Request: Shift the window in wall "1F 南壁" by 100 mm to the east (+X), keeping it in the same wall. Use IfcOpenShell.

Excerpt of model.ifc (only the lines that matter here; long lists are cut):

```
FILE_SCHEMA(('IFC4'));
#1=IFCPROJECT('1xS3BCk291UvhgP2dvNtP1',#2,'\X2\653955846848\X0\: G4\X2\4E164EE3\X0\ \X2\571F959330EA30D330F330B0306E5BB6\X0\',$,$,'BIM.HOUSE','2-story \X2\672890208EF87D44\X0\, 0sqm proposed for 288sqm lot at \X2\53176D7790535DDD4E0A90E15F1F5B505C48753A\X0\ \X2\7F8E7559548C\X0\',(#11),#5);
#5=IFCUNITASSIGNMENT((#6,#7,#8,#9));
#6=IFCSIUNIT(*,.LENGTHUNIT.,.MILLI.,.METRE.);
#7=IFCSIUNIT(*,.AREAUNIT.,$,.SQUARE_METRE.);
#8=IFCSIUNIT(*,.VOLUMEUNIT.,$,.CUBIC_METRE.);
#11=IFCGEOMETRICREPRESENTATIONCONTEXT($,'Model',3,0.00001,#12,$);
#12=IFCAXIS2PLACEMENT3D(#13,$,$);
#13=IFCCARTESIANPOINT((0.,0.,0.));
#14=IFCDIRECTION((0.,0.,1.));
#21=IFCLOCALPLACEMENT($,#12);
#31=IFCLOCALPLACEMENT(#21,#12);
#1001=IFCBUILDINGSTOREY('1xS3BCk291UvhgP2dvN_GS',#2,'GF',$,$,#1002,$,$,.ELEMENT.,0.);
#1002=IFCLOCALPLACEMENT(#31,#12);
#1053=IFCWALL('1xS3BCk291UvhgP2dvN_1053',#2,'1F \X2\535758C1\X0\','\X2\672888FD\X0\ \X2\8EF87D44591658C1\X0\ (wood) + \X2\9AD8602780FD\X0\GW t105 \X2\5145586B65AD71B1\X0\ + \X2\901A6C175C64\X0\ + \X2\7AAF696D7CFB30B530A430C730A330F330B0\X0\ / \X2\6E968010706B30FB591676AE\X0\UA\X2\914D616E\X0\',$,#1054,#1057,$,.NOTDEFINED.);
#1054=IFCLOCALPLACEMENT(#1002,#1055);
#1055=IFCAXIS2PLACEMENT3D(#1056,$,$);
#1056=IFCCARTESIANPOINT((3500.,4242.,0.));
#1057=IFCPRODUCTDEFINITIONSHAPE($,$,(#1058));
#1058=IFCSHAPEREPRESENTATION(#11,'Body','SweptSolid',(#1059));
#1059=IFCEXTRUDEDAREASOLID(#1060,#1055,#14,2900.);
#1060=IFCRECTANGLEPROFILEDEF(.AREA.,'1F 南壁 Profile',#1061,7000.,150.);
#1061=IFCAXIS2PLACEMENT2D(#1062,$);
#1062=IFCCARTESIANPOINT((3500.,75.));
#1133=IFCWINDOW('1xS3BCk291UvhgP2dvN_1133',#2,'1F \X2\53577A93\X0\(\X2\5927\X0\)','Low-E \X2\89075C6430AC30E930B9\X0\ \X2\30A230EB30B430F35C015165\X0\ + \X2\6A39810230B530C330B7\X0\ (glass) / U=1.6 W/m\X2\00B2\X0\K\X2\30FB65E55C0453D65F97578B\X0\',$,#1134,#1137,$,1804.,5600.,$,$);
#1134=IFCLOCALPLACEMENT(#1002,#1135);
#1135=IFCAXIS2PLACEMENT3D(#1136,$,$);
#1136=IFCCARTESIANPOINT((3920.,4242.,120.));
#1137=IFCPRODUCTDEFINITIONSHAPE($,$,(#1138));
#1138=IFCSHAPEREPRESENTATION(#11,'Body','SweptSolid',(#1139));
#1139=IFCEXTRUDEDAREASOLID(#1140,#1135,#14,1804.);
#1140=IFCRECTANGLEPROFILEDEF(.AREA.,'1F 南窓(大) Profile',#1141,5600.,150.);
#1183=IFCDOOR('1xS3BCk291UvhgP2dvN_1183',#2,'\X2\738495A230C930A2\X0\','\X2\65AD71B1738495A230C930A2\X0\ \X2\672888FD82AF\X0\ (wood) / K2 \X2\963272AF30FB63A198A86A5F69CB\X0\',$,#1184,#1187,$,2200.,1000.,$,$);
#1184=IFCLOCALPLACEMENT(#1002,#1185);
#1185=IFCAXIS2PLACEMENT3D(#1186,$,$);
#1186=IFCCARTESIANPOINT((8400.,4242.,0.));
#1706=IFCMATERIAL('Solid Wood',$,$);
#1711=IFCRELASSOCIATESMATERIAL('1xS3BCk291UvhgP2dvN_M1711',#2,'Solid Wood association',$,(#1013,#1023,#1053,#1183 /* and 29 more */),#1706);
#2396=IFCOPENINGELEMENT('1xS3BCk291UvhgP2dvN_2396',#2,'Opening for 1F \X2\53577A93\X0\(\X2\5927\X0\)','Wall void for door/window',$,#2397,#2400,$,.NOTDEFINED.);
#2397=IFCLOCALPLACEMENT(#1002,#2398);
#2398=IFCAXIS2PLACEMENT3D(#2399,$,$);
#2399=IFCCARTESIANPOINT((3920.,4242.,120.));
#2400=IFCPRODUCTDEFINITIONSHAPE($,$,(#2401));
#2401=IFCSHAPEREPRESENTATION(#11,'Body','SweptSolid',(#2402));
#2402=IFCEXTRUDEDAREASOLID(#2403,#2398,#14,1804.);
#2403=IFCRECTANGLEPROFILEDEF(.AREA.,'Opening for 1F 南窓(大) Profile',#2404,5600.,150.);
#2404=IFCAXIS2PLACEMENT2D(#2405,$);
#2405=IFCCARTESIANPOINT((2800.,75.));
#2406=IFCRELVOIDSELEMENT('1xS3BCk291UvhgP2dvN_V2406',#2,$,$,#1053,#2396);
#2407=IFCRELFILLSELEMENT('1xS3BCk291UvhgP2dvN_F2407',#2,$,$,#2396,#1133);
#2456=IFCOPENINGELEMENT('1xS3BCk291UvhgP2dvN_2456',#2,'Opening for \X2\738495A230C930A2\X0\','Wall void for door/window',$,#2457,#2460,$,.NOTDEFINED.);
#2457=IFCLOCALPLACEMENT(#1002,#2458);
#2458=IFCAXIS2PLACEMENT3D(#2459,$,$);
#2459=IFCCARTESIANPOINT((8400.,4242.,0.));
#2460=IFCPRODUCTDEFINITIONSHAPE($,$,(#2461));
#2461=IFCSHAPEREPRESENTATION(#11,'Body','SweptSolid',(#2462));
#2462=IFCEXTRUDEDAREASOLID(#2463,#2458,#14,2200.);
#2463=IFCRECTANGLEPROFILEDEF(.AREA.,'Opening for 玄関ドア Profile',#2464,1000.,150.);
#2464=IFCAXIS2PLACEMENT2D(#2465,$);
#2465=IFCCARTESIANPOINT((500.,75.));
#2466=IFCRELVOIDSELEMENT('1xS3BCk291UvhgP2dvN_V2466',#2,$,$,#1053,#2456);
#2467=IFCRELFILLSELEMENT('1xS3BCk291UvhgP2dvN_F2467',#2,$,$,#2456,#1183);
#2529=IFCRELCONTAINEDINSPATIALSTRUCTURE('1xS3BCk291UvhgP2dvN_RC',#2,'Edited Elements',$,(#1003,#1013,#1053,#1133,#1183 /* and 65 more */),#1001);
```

```python
import ifcopenshell
import ifcopenshell.api.geometry
import ifcopenshell.util.placement

model = ifcopenshell.open("model.ifc")

window = model.by_guid("1xS3BCk291UvhgP2dvN_1133")
opening = window.FillsVoids[0].RelatingOpeningElement
wall = opening.VoidsElements[0].RelatingBuildingElement

wall_matrix = ifcopenshell.util.placement.get_local_placement(wall.ObjectPlacement)
shift = wall_matrix[:3, 0] * 100.0
before = ifcopenshell.util.placement.get_local_placement(window.ObjectPlacement)[:3, 3].copy()

# The window is not placed relative to its opening, so move both.
for product in (opening, window):
    matrix = ifcopenshell.util.placement.get_local_placement(product.ObjectPlacement)
    matrix[:3, 3] += shift
    ifcopenshell.api.geometry.edit_object_placement(model, product=product, matrix=matrix, is_si=False)

after = ifcopenshell.util.placement.get_local_placement(window.ObjectPlacement)[:3, 3]
print("window moved by", (after - before).round(3) + 0.0)

model.write("model-out.ifc")
```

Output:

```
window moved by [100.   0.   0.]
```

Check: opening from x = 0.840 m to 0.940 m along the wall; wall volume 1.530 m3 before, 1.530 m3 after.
